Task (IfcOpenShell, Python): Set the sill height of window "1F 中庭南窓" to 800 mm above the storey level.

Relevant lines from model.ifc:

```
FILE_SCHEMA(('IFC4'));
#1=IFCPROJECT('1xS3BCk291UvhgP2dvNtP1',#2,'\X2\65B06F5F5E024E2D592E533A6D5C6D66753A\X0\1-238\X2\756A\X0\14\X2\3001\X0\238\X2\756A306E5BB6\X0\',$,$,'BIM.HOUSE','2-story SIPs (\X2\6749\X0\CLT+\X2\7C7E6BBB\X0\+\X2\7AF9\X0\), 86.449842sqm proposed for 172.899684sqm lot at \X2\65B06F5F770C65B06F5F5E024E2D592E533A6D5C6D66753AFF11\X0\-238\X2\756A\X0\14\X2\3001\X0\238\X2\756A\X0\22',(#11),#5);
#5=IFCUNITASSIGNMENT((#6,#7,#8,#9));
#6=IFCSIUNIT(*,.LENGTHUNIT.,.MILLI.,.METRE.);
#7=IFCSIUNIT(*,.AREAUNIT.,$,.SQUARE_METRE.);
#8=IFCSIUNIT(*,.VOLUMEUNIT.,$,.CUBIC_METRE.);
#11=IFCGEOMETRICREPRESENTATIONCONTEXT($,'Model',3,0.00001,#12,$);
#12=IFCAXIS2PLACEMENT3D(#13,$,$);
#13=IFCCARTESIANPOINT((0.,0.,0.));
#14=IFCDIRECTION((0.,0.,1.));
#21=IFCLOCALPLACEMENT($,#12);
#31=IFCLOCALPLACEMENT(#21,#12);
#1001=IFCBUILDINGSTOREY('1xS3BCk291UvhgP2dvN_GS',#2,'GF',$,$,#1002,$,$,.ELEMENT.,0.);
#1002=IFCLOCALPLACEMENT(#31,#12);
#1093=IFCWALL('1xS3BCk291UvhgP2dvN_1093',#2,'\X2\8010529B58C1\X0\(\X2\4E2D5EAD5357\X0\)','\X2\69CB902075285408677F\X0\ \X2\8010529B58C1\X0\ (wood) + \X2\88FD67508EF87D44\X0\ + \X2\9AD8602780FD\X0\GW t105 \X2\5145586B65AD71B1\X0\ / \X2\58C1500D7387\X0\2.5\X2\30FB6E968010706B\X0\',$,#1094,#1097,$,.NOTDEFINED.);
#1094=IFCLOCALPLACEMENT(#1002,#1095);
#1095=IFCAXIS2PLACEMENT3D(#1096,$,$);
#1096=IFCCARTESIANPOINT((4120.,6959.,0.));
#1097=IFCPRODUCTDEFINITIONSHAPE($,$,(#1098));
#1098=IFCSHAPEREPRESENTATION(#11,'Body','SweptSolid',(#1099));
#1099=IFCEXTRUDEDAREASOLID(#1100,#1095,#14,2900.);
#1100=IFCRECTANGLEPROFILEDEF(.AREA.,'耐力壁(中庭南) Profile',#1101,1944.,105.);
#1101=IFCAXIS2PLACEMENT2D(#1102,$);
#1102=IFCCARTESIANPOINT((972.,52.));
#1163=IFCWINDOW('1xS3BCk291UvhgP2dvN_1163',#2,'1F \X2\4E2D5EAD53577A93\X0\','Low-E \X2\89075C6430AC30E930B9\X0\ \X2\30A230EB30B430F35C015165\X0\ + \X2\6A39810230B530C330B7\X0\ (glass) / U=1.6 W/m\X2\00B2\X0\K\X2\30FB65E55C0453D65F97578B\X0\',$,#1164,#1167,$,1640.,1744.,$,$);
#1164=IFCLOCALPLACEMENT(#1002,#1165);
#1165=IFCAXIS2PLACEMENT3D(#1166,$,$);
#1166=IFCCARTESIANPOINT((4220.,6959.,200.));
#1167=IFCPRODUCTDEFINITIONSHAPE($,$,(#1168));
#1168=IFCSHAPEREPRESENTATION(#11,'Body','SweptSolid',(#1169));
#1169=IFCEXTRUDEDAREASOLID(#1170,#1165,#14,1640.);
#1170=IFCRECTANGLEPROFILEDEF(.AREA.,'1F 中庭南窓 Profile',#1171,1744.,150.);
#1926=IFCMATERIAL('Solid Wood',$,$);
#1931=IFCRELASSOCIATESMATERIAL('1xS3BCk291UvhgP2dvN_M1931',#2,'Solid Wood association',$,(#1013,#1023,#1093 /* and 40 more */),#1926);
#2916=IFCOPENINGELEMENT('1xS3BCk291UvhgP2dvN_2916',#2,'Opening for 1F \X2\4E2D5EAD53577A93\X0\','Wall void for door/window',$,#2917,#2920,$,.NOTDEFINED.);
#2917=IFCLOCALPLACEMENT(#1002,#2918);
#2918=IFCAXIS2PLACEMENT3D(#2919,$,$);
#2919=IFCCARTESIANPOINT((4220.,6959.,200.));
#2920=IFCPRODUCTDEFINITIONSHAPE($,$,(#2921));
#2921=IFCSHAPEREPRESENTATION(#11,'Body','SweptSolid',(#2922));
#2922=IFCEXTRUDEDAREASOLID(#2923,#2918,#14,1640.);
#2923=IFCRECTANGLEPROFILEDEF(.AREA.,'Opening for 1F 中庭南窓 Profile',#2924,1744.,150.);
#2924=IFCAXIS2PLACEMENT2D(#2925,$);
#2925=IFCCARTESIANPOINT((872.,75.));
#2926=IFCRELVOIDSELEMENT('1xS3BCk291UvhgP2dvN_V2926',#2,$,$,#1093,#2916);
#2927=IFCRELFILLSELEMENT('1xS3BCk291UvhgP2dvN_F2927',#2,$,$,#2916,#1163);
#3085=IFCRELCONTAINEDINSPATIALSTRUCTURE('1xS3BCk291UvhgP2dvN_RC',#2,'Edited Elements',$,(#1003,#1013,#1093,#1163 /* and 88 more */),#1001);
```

```python
import numpy as np
import ifcopenshell
import ifcopenshell.api.geometry
import ifcopenshell.geom
import ifcopenshell.util.element
import ifcopenshell.util.placement
import ifcopenshell.util.shape
import ifcopenshell.util.unit

model = ifcopenshell.open("model.ifc")
unit_scale = ifcopenshell.util.unit.calculate_unit_scale(model)

window = model.by_guid("1xS3BCk291UvhgP2dvN_1163")
opening = window.FillsVoids[0].RelatingOpeningElement
storey = ifcopenshell.util.element.get_container(window, ifc_class="IfcBuildingStorey")
level = ifcopenshell.util.placement.get_local_placement(storey.ObjectPlacement)[2, 3]

# The opening's origin need not be at the sill, so measure its lowest point.
shape = ifcopenshell.geom.create_shape(ifcopenshell.geom.settings(), opening)
bottom = ifcopenshell.util.shape.get_shape_bottom_elevation(shape, shape.geometry) / unit_scale
dz = level + 800.0 - bottom

shift = np.array([0.0, 0.0, dz])
# The window is not placed relative to its opening, so move both.
for product in (opening, window):
    matrix = ifcopenshell.util.placement.get_local_placement(product.ObjectPlacement)
    matrix[:3, 3] += shift
    ifcopenshell.api.geometry.edit_object_placement(model, product=product, matrix=matrix, is_si=False)

print(f"moved by {dz * unit_scale:+.3f} m")

model.write("model_updated.ifc")
```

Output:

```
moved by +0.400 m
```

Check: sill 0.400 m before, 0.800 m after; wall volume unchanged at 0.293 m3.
